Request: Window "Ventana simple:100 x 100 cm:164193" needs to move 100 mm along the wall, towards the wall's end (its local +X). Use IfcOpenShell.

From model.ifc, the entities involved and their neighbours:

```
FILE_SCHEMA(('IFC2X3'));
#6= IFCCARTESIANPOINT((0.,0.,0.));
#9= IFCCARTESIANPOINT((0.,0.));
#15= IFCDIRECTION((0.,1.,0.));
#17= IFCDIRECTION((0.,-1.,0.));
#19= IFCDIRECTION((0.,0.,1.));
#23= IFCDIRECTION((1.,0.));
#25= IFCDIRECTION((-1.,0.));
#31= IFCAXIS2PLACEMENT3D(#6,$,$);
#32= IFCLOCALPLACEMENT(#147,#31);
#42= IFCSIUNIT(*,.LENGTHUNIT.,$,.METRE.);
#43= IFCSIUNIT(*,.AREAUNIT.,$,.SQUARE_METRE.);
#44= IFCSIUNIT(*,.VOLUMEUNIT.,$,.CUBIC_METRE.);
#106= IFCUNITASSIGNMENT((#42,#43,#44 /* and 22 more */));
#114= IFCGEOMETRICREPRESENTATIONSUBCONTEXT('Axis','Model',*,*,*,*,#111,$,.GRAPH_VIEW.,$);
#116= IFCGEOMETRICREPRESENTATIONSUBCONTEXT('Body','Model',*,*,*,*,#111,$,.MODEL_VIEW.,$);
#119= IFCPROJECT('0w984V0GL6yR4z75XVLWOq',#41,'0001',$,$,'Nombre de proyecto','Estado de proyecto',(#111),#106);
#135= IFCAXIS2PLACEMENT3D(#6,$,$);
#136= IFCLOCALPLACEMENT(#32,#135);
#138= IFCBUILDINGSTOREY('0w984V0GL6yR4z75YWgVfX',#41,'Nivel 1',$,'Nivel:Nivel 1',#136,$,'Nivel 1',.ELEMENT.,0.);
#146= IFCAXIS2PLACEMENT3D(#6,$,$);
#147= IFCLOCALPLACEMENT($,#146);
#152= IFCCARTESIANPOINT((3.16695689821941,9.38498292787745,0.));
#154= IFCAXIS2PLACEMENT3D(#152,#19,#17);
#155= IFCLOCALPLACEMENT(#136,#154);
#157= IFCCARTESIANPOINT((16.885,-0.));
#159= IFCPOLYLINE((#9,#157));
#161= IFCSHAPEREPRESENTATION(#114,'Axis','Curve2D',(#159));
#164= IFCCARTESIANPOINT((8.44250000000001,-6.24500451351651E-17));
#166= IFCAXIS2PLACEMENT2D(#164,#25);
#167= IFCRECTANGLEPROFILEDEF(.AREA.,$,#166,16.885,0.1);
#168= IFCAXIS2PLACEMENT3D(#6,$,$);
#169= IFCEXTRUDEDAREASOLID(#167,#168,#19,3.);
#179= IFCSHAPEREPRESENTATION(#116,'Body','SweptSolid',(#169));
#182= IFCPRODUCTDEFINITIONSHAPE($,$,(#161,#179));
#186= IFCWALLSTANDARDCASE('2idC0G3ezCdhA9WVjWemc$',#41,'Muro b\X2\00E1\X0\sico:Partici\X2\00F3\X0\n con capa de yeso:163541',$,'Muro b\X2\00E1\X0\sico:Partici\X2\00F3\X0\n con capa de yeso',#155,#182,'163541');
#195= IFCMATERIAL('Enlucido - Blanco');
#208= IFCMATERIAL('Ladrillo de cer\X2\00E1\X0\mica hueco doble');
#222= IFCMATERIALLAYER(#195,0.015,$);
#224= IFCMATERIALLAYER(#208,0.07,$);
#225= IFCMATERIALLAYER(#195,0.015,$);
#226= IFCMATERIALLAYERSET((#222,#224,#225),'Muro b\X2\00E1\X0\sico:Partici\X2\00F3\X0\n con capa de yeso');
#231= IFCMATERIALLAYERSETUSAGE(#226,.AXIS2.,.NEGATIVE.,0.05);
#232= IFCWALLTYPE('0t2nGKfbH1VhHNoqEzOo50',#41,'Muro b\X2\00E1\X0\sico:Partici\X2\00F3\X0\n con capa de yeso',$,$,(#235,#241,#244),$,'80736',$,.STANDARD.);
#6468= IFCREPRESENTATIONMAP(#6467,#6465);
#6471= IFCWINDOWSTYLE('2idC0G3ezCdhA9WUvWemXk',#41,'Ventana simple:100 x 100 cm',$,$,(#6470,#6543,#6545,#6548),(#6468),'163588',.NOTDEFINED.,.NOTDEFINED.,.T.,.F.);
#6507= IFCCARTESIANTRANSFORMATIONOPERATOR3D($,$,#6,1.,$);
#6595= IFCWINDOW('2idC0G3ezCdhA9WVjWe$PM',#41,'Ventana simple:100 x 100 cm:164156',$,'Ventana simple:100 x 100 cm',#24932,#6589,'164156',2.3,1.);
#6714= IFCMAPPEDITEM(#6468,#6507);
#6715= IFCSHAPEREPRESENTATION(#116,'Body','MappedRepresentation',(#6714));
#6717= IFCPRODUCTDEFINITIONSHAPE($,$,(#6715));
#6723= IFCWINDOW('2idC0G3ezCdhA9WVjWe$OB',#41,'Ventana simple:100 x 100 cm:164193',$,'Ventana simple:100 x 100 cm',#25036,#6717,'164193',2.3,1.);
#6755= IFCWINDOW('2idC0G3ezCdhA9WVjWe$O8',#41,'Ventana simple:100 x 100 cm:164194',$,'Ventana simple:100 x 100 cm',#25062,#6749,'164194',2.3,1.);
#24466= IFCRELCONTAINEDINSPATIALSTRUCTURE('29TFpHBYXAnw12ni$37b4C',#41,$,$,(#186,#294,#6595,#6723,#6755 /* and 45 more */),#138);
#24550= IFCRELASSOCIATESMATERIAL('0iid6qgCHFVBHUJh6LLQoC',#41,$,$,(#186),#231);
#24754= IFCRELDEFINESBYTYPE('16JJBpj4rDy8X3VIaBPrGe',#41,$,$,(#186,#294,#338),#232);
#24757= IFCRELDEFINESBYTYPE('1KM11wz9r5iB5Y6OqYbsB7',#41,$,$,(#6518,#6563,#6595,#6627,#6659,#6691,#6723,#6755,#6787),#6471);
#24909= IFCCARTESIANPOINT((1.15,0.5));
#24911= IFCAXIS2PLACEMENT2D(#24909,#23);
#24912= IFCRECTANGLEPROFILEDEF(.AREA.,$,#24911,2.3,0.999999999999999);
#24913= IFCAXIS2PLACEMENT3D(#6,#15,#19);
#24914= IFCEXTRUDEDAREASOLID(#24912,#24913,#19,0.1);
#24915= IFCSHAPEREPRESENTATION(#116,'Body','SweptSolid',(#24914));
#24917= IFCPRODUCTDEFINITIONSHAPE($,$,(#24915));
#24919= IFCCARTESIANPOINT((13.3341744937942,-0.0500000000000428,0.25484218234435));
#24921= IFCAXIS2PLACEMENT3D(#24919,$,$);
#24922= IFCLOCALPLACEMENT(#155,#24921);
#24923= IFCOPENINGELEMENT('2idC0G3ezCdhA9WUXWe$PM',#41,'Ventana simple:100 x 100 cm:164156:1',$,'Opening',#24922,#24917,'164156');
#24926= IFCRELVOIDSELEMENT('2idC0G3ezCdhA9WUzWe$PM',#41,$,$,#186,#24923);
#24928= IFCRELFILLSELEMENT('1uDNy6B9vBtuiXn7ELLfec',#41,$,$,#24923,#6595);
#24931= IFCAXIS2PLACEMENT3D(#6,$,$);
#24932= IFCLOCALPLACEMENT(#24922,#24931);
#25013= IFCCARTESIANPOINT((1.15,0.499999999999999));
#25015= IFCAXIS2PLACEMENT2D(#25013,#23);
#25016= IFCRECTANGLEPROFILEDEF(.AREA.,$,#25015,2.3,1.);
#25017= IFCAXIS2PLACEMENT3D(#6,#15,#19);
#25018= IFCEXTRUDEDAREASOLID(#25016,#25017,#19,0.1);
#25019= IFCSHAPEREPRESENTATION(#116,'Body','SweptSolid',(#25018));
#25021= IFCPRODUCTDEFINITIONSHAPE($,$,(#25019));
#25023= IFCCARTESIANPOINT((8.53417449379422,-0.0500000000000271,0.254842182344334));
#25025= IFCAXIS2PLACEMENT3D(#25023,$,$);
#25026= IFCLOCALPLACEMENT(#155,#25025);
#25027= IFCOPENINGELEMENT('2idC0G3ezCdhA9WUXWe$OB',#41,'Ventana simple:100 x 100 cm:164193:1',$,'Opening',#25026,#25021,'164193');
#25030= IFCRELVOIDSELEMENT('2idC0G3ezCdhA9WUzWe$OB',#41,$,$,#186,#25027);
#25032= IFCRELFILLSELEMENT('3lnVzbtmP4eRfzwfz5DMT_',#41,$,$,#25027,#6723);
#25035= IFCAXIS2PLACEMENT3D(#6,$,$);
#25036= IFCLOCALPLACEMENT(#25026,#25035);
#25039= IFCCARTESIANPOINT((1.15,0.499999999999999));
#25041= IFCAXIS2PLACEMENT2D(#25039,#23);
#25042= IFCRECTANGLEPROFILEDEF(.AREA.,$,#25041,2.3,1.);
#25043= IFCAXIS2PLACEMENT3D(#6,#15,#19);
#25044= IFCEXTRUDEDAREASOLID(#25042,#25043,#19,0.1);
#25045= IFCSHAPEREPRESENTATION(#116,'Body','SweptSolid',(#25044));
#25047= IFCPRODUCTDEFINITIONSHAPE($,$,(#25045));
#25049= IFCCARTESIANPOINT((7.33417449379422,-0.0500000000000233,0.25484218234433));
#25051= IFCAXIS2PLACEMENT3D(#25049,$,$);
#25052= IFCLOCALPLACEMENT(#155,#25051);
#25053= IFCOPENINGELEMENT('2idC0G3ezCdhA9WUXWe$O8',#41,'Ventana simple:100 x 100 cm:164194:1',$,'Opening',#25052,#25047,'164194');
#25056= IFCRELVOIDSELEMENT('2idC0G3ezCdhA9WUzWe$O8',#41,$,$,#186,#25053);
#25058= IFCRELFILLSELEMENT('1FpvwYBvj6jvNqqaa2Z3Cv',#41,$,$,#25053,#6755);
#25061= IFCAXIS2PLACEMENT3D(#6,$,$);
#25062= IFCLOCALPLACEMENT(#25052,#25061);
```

```python
import ifcopenshell
import ifcopenshell.api.geometry
import ifcopenshell.util.placement
import ifcopenshell.util.unit

model = ifcopenshell.open("model.ifc")
unit_scale = ifcopenshell.util.unit.calculate_unit_scale(model)

window = model.by_guid("2idC0G3ezCdhA9WVjWe$OB")
opening = window.FillsVoids[0].RelatingOpeningElement
wall = opening.VoidsElements[0].RelatingBuildingElement

wall_matrix = ifcopenshell.util.placement.get_local_placement(wall.ObjectPlacement)
shift = wall_matrix[:3, 0] * 0.1 / unit_scale
before = ifcopenshell.util.placement.get_local_placement(window.ObjectPlacement)[:3, 3].copy()

# The window is placed relative to its opening, so it follows when the opening moves.
matrix = ifcopenshell.util.placement.get_local_placement(opening.ObjectPlacement)
matrix[:3, 3] += shift
ifcopenshell.api.geometry.edit_object_placement(
    model, product=opening, matrix=matrix, is_si=False, should_transform_children=True
)

after = ifcopenshell.util.placement.get_local_placement(window.ObjectPlacement)[:3, 3]
print("window moved by", (after - before).round(3) + 0.0)

model.write("model_updated.ifc")
```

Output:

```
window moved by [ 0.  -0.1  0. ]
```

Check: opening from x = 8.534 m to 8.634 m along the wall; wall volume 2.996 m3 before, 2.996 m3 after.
